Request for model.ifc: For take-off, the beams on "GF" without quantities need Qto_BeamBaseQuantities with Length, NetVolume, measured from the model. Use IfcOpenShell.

First a look at what the model holds.

```python
import ifcopenshell
import ifcopenshell.util.element
import ifcopenshell.util.unit

model = ifcopenshell.open("model.ifc")
print(model.schema)
for unit_type in ("LENGTHUNIT", "AREAUNIT", "VOLUMEUNIT"):
    print(unit_type, ifcopenshell.util.unit.calculate_unit_scale(model, unit_type))
storey = next(s for s in model.by_type("IfcBuildingStorey") if s.Name == "GF")
beams = [e for e in ifcopenshell.util.element.get_decomposition(storey) if e.is_a("IfcBeam")]
for e in sorted(beams, key=lambda e: e.id()):
    print(e.id(), e.is_a(), e.Name, list(ifcopenshell.util.element.get_psets(e, qtos_only=True)), sep=" | ")
```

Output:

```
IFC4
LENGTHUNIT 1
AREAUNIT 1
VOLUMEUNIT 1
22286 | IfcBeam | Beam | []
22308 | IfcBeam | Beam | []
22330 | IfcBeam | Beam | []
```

```python
import ifcopenshell
import ifcopenshell.api.pset
import ifcopenshell.geom
import ifcopenshell.util.element
import ifcopenshell.util.shape
import ifcopenshell.util.unit

model = ifcopenshell.open("model.ifc")
unit_scale = ifcopenshell.util.unit.calculate_unit_scale(model)
volume_scale = ifcopenshell.util.unit.calculate_unit_scale(model, "VOLUMEUNIT")
settings = ifcopenshell.geom.settings()

storey = next(s for s in model.by_type("IfcBuildingStorey") if s.Name == "GF")
beams = [e for e in ifcopenshell.util.element.get_decomposition(storey) if e.is_a("IfcBeam")]

for e in sorted(beams, key=lambda e: e.id()):
    if ifcopenshell.util.element.get_psets(e, qtos_only=True, should_inherit=False):
        continue
    # Geometry comes back in metres, in the element's own axes.
    shape = ifcopenshell.geom.create_shape(settings, e)
    values = {
        "Length": ifcopenshell.util.shape.get_max_xyz(shape.geometry) / unit_scale,
        "NetVolume": ifcopenshell.util.shape.get_volume(shape.geometry) / volume_scale,
    }
    qto = ifcopenshell.api.pset.add_qto(model, product=e, name="Qto_BeamBaseQuantities")
    ifcopenshell.api.pset.edit_qto(model, qto=qto, properties=values)
    print(e.id(), {k: round(v, 3) for k, v in values.items()})

model.write("model_rev.ifc")
```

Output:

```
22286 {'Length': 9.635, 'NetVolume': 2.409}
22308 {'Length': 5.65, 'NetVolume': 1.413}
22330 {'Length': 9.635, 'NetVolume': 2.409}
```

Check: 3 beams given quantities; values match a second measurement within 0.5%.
